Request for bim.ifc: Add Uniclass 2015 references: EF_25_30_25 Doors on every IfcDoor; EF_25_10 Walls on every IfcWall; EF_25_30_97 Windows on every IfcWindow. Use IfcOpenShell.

First a look at what the model holds.

```python
import ifcopenshell

model = ifcopenshell.open("bim.ifc")
print(model.schema)
print("classifications:", [c.Name for c in model.by_type("IfcClassification")])
for ifc_class in ("IfcDoor", "IfcRoof", "IfcStair", "IfcWall", "IfcWindow"):
    print(ifc_class, len(model.by_type(ifc_class)))
```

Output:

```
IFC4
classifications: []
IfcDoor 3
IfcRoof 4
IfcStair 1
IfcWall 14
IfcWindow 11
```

```python
import ifcopenshell
import ifcopenshell.api.classification

model = ifcopenshell.open("bim.ifc")

system = ifcopenshell.api.classification.add_classification(model, classification="Uniclass 2015")

codes = {
    "IfcDoor": ("EF_25_30_25", "Doors"),
    "IfcWall": ("EF_25_10", "Walls"),
    "IfcWindow": ("EF_25_30_97", "Windows"),
}
for ifc_class, (code, name) in codes.items():
    products = model.by_type(ifc_class)
    ifcopenshell.api.classification.add_reference(
        model, products=products, classification=system, identification=code, name=name
    )
    print(code, len(products))

model.write("bim_v2.ifc")
```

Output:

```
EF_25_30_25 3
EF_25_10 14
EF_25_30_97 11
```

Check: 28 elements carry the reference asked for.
